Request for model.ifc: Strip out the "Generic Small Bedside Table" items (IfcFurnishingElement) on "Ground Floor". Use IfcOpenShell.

First a look at what the model holds.

```python
import ifcopenshell
import ifcopenshell.util.element

model = ifcopenshell.open("model.ifc")
print(model.schema)
storey = next(s for s in model.by_type("IfcBuildingStorey") if s.Name == "Ground Floor")
furniture = [e for e in ifcopenshell.util.element.get_decomposition(storey) if e.is_a("IfcFurnishingElement")]
seen = {}
for e in furniture:
    element_type = ifcopenshell.util.element.get_type(e)
    name = element_type.Name if element_type not in (None, e) else None
    seen[name] = seen.get(name, 0) + 1
for name, count in sorted(seen.items(), key=str):
    print(count, "x", name)
```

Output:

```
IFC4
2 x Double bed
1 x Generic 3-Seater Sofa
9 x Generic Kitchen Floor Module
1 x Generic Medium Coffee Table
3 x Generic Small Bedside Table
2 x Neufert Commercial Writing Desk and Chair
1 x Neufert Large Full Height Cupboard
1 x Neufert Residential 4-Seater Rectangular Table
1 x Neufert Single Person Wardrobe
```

```python
import ifcopenshell
import ifcopenshell.api.root
import ifcopenshell.util.element

model = ifcopenshell.open("model.ifc")

storey = next(s for s in model.by_type("IfcBuildingStorey") if s.Name == "Ground Floor")
furniture = [e for e in ifcopenshell.util.element.get_decomposition(storey) if e.is_a("IfcFurnishingElement")]
targets = [e for e in furniture if (t := ifcopenshell.util.element.get_type(e)) not in (None, e) and t.Name == "Generic Small Bedside Table"]

for e in targets:
    ifcopenshell.api.root.remove_product(model, product=e)
print(len(targets), "removed")

model.write("model_rev.ifc")
```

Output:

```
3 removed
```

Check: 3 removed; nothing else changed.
